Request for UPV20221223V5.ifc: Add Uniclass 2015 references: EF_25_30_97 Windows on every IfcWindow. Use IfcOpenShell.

First a look at what the model holds.

```python
import ifcopenshell

model = ifcopenshell.open("UPV20221223V5.ifc")
print(model.schema)
print("classifications:", [c.Name for c in model.by_type("IfcClassification")])
for ifc_class in ("IfcDoor", "IfcRoof", "IfcStair", "IfcWall", "IfcWindow"):
    print(ifc_class, len(model.by_type(ifc_class)))
```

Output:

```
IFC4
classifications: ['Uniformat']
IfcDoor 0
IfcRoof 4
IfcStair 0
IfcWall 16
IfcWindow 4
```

```python
import ifcopenshell
import ifcopenshell.api.classification

model = ifcopenshell.open("UPV20221223V5.ifc")

system = ifcopenshell.api.classification.add_classification(model, classification="Uniclass 2015")

codes = {
    "IfcWindow": ("EF_25_30_97", "Windows"),
}
for ifc_class, (code, name) in codes.items():
    products = model.by_type(ifc_class)
    ifcopenshell.api.classification.add_reference(
        model, products=products, classification=system, identification=code, name=name
    )
    print(code, len(products))

model.write("UPV20221223V5-out.ifc")
```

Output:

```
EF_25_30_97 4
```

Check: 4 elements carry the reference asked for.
